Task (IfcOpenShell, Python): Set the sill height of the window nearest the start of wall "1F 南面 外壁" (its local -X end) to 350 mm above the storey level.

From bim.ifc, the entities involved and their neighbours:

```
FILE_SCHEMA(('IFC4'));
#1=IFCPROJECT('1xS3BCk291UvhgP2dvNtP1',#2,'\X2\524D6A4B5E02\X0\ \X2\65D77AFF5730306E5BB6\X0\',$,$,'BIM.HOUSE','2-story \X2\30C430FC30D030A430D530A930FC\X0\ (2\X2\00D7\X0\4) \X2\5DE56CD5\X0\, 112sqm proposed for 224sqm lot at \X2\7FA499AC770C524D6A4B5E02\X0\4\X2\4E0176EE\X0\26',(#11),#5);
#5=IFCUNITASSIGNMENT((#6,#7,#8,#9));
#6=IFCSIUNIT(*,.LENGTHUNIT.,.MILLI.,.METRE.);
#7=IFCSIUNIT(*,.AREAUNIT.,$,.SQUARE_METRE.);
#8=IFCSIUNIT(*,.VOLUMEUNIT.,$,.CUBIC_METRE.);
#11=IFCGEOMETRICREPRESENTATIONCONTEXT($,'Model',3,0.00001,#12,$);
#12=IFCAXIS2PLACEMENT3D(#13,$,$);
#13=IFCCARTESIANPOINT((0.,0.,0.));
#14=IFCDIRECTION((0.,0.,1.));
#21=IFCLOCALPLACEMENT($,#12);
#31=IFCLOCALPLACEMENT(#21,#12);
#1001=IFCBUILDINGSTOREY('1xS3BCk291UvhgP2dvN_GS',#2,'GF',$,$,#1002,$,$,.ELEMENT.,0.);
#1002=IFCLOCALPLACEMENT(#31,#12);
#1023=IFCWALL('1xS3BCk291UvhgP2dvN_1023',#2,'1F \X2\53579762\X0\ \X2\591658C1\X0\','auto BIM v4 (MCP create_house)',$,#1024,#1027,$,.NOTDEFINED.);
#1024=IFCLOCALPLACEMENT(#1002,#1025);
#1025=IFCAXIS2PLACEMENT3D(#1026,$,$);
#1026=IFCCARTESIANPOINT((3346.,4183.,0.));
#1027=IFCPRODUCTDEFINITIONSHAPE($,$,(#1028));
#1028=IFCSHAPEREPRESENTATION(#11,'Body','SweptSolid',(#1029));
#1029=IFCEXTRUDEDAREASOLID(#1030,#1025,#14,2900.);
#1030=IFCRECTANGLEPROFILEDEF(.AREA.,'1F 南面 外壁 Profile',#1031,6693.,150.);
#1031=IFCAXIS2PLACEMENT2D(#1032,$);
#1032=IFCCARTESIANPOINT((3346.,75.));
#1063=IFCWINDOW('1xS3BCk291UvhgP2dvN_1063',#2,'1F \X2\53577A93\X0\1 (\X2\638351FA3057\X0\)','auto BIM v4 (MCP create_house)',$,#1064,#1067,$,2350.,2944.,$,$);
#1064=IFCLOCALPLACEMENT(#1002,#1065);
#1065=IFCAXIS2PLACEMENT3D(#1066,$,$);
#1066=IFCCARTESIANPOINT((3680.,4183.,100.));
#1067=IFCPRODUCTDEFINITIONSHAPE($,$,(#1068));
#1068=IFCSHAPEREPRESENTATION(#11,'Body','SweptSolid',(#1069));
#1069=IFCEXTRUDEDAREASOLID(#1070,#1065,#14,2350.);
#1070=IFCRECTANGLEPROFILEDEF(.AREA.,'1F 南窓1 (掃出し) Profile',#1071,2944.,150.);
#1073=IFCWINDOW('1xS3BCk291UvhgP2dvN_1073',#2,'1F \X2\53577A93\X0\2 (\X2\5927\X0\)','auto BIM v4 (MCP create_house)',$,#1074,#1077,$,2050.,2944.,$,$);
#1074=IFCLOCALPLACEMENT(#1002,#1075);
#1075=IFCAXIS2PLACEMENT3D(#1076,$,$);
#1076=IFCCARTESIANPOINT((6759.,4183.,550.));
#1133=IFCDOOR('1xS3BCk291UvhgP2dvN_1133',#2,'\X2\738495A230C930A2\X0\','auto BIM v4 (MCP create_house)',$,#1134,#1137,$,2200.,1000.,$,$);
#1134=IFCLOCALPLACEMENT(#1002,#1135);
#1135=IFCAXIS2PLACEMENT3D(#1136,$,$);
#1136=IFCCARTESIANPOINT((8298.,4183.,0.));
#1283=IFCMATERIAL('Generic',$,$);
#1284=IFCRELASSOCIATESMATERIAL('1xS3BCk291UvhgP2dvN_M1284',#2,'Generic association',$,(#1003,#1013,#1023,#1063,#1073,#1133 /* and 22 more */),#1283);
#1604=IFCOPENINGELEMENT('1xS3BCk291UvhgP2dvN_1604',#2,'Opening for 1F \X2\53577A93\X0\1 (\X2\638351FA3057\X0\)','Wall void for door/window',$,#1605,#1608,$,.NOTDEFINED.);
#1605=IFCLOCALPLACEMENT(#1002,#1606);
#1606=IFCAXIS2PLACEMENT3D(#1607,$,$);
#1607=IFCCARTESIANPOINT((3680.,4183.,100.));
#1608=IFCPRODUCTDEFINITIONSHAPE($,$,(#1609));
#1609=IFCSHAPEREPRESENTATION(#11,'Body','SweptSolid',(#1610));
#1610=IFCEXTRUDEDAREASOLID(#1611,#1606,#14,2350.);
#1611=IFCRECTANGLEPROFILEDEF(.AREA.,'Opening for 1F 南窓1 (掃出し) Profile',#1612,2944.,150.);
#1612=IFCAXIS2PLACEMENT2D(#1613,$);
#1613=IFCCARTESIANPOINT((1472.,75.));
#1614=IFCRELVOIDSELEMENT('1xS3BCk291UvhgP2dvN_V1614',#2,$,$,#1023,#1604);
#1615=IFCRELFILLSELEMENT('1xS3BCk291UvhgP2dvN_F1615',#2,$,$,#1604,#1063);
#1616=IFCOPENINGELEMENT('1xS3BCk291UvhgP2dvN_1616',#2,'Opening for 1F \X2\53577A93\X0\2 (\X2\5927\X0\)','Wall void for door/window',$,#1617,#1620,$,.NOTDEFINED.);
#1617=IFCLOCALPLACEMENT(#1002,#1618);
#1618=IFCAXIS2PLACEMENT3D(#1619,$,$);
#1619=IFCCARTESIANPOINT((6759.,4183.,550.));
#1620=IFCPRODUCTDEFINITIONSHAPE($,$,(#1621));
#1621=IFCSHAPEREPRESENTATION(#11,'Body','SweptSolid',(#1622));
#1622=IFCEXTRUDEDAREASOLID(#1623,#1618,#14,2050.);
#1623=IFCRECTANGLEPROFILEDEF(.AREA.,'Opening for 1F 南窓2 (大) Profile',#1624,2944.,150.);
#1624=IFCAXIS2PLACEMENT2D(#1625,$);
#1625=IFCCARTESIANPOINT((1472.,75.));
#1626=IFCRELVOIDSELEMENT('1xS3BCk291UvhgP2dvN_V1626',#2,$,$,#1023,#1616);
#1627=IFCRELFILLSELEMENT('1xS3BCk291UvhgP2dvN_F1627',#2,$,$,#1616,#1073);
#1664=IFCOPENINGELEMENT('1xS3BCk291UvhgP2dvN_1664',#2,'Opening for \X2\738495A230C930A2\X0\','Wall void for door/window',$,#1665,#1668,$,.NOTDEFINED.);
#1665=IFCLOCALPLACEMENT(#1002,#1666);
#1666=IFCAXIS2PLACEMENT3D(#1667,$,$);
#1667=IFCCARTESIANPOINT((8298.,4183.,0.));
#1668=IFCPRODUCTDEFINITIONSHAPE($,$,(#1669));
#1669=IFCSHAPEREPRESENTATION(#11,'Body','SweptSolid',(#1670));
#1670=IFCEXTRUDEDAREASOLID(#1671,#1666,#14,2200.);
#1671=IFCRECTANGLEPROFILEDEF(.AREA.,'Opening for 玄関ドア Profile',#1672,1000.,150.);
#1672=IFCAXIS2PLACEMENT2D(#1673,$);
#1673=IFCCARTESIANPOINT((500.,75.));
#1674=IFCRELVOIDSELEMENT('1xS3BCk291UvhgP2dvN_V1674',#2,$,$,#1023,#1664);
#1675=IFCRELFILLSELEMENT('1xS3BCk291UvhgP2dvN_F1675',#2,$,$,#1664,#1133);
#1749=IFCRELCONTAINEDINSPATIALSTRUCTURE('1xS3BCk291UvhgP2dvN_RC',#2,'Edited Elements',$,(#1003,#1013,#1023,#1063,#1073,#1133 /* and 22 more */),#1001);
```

```python
import numpy as np
import ifcopenshell
import ifcopenshell.api.geometry
import ifcopenshell.geom
import ifcopenshell.util.element
import ifcopenshell.util.placement
import ifcopenshell.util.shape
import ifcopenshell.util.unit

model = ifcopenshell.open("bim.ifc")
unit_scale = ifcopenshell.util.unit.calculate_unit_scale(model)

window = model.by_guid("1xS3BCk291UvhgP2dvN_1063")
opening = window.FillsVoids[0].RelatingOpeningElement
storey = ifcopenshell.util.element.get_container(window, ifc_class="IfcBuildingStorey")
level = ifcopenshell.util.placement.get_local_placement(storey.ObjectPlacement)[2, 3]

# The opening's origin need not be at the sill, so measure its lowest point.
shape = ifcopenshell.geom.create_shape(ifcopenshell.geom.settings(), opening)
bottom = ifcopenshell.util.shape.get_shape_bottom_elevation(shape, shape.geometry) / unit_scale
dz = level + 0.35 / unit_scale - bottom

shift = np.array([0.0, 0.0, dz])
# The window is not placed relative to its opening, so move both.
for product in (opening, window):
    matrix = ifcopenshell.util.placement.get_local_placement(product.ObjectPlacement)
    matrix[:3, 3] += shift
    ifcopenshell.api.geometry.edit_object_placement(model, product=product, matrix=matrix, is_si=False)

print(f"moved by {dz * unit_scale:+.3f} m")

model.write("bim_edited.ifc")
```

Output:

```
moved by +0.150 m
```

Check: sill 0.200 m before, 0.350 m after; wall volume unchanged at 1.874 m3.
